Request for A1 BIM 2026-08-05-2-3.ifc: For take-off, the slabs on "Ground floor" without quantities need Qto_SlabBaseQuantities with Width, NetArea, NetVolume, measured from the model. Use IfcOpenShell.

First a look at what the model holds.

```python
import ifcopenshell
import ifcopenshell.util.element
import ifcopenshell.util.unit

model = ifcopenshell.open("A1 BIM 2026-08-05-2-3.ifc")
print(model.schema)
for unit_type in ("LENGTHUNIT", "AREAUNIT", "VOLUMEUNIT"):
    print(unit_type, ifcopenshell.util.unit.calculate_unit_scale(model, unit_type))
storey = next(s for s in model.by_type("IfcBuildingStorey") if s.Name == "Ground floor")
slabs = [e for e in ifcopenshell.util.element.get_decomposition(storey) if e.is_a("IfcSlab")]
for e in sorted(slabs, key=lambda e: e.id()):
    print(e.id(), e.is_a(), e.Name, list(ifcopenshell.util.element.get_psets(e, qtos_only=True)), sep=" | ")
```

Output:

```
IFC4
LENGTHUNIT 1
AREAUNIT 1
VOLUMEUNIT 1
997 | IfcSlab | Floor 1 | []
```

```python
import ifcopenshell
import ifcopenshell.api.pset
import ifcopenshell.geom
import ifcopenshell.util.element
import ifcopenshell.util.shape
import ifcopenshell.util.unit

model = ifcopenshell.open("A1 BIM 2026-08-05-2-3.ifc")
unit_scale = ifcopenshell.util.unit.calculate_unit_scale(model)
area_scale = ifcopenshell.util.unit.calculate_unit_scale(model, "AREAUNIT")
volume_scale = ifcopenshell.util.unit.calculate_unit_scale(model, "VOLUMEUNIT")
settings = ifcopenshell.geom.settings()

storey = next(s for s in model.by_type("IfcBuildingStorey") if s.Name == "Ground floor")
slabs = [e for e in ifcopenshell.util.element.get_decomposition(storey) if e.is_a("IfcSlab")]

for e in sorted(slabs, key=lambda e: e.id()):
    if ifcopenshell.util.element.get_psets(e, qtos_only=True, should_inherit=False):
        continue
    # Geometry comes back in metres, in the element's own axes.
    shape = ifcopenshell.geom.create_shape(settings, e)
    values = {
        "Width": ifcopenshell.util.shape.get_z(shape.geometry) / unit_scale,
        "NetArea": ifcopenshell.util.shape.get_footprint_area(shape.geometry) / area_scale,
        "NetVolume": ifcopenshell.util.shape.get_volume(shape.geometry) / volume_scale,
    }
    qto = ifcopenshell.api.pset.add_qto(model, product=e, name="Qto_SlabBaseQuantities")
    ifcopenshell.api.pset.edit_qto(model, qto=qto, properties=values)
    print(e.id(), {k: round(v, 3) for k, v in values.items()})

model.write("A1 BIM 2026-08-05-2-3_edited.ifc")
```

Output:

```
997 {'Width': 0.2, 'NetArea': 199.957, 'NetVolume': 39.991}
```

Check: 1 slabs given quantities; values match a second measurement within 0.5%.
